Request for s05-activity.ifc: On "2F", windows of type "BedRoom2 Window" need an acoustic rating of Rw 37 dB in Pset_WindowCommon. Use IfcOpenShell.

First a look at what the model holds.

```python
import ifcopenshell
import ifcopenshell.util.element

model = ifcopenshell.open("s05-activity.ifc")
print(model.schema)
storey = next(s for s in model.by_type("IfcBuildingStorey") if s.Name == "2F")
windows = [e for e in ifcopenshell.util.element.get_decomposition(storey) if e.is_a("IfcWindow")]
seen = {}
for e in windows:
    element_type = ifcopenshell.util.element.get_type(e)
    key = (element_type.Name if element_type != e and element_type else None, ifcopenshell.util.element.get_pset(e, "Pset_WindowCommon", "AcousticRating"))
    seen[key] = seen.get(key, 0) + 1
for (name, value), count in sorted(seen.items(), key=str):
    print(count, "x", name, "|", value)
```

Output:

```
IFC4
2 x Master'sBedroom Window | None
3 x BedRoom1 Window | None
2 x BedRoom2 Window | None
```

```python
import ifcopenshell
import ifcopenshell.api.pset
import ifcopenshell.util.element

model = ifcopenshell.open("s05-activity.ifc")

storey = next(s for s in model.by_type("IfcBuildingStorey") if s.Name == "2F")
windows = [e for e in ifcopenshell.util.element.get_decomposition(storey) if e.is_a("IfcWindow")]

count = 0
for e in windows:
    element_type = ifcopenshell.util.element.get_type(e)
    if element_type in (None, e) or element_type.Name != "BedRoom2 Window":
        continue
    # add_pset returns the element's existing set when there is one.
    pset = ifcopenshell.api.pset.add_pset(model, product=e, name="Pset_WindowCommon")
    ifcopenshell.api.pset.edit_pset(model, pset=pset, properties={"AcousticRating": "Rw 37 dB"})
    count += 1

print(count, "windows updated")

model.write("s05-activity_updated.ifc")
```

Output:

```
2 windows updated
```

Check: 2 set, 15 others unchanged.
